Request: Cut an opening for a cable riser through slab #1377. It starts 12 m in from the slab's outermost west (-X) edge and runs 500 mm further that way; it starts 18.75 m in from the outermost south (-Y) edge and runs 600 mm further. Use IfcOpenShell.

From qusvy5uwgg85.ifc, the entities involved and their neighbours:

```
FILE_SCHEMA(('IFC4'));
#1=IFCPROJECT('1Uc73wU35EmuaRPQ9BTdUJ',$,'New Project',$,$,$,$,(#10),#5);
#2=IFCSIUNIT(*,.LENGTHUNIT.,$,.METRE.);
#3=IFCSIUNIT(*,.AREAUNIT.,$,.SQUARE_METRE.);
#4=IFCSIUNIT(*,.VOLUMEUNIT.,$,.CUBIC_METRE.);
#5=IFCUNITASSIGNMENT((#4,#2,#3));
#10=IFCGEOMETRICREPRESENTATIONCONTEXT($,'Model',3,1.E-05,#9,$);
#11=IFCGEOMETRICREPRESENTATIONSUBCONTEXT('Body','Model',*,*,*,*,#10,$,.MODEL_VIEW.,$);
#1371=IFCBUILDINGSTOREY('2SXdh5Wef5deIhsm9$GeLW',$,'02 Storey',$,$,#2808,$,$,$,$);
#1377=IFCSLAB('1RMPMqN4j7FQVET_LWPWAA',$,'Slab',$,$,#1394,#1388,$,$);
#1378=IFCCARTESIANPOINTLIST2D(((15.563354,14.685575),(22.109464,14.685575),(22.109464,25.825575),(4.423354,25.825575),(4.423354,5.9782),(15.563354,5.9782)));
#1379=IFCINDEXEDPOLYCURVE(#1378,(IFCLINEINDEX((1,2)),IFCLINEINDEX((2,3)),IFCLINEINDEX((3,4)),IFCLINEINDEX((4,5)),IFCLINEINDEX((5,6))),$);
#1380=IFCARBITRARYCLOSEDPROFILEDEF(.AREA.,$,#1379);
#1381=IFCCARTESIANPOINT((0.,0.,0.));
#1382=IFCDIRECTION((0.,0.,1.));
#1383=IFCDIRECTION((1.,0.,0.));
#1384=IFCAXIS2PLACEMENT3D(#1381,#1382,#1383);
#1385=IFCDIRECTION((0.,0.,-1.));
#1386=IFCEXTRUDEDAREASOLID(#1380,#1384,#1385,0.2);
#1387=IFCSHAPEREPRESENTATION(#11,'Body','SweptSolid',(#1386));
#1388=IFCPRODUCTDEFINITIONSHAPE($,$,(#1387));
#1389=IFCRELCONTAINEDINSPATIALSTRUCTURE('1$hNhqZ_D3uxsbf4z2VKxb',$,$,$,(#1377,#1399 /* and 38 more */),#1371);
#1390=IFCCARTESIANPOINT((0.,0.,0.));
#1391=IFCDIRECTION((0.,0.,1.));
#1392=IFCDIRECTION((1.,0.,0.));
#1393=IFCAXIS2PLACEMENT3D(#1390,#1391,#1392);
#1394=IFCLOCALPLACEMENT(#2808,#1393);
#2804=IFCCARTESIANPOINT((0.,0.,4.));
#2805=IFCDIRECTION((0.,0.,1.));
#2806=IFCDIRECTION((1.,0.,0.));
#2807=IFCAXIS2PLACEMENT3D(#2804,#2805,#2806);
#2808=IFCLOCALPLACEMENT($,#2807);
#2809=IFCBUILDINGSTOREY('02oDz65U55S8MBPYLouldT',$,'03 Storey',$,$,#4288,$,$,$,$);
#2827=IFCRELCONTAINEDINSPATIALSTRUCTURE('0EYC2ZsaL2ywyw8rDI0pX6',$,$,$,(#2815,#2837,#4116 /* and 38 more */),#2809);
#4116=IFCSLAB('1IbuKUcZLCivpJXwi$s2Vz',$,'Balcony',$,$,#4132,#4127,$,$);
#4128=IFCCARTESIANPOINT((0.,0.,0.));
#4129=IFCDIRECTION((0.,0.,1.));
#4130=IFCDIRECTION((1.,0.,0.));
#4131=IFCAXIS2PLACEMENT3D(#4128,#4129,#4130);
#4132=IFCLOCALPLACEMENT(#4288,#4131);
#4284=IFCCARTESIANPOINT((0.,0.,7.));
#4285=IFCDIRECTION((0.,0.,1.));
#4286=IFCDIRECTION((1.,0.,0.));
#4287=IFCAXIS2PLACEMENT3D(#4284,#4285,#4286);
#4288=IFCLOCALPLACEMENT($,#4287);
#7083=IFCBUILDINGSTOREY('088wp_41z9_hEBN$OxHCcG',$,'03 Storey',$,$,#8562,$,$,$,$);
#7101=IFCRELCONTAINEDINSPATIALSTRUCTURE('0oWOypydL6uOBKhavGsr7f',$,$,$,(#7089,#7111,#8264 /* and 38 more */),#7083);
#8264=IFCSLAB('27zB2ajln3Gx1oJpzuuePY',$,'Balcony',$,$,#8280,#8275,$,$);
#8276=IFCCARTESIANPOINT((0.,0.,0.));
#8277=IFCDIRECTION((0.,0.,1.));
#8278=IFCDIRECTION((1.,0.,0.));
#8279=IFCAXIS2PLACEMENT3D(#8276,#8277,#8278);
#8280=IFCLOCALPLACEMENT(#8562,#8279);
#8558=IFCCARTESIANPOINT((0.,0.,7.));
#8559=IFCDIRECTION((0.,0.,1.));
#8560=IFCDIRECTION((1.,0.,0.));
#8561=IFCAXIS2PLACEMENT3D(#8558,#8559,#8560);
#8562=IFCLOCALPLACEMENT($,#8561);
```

```python
import numpy as np
import ifcopenshell
import ifcopenshell.api.feature
import ifcopenshell.api.geometry
import ifcopenshell.api.root
import ifcopenshell.geom
import ifcopenshell.util.placement
import ifcopenshell.util.representation
import ifcopenshell.util.shape
import ifcopenshell.util.unit

model = ifcopenshell.open("qusvy5uwgg85.ifc")
unit_scale = ifcopenshell.util.unit.calculate_unit_scale(model)
settings = ifcopenshell.geom.settings()


def volume(element):
    """Net volume in cubic metres, openings subtracted."""
    shape = ifcopenshell.geom.create_shape(settings, element)
    return ifcopenshell.util.shape.get_volume(shape.geometry)


slab = model.by_guid("1RMPMqN4j7FQVET_LWPWAA")
before = volume(slab)

# Extent in the slab's own axes, in metres. The edges named are its -X and -Y sides.
slab_shape = ifcopenshell.geom.create_shape(settings, slab)
vertices = ifcopenshell.util.shape.get_vertices(slab_shape.geometry)
x_min, y_min, bottom = vertices.min(axis=0)
top = vertices[:, 2].max()

opening = ifcopenshell.api.root.create_entity(model, ifc_class="IfcOpeningElement", name="Cable riser opening", predefined_type="OPENING")
context = ifcopenshell.util.representation.get_context(model, "Model", "Body", "MODEL_VIEW")
width, depth = 0.5, 0.6
outline = [(0.0, 0.0), (width, 0.0), (width, depth), (0.0, depth), (0.0, 0.0)]
# Overshoot both faces by 50 mm so the cut is clean.
shape = ifcopenshell.api.geometry.add_slab_representation(
    model, context=context, depth=top - bottom + 0.1, polyline=outline
)
ifcopenshell.api.geometry.assign_representation(model, product=opening, representation=shape)

matrix = ifcopenshell.util.placement.get_local_placement(slab.ObjectPlacement)
matrix[:, 3] = matrix @ np.append(np.array([x_min + 12, y_min + 18.75, bottom - 0.05]) / unit_scale, 1.0)
ifcopenshell.api.geometry.edit_object_placement(model, product=opening, matrix=matrix, is_si=False)
ifcopenshell.api.feature.add_feature(model, feature=opening, element=slab)

after = volume(slab)

print(f"slab volume {before:.3f} -> {after:.3f} m3")

model.write("qusvy5uwgg85_v2.ifc")
```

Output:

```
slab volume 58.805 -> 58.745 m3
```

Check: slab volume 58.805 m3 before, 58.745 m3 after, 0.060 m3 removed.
